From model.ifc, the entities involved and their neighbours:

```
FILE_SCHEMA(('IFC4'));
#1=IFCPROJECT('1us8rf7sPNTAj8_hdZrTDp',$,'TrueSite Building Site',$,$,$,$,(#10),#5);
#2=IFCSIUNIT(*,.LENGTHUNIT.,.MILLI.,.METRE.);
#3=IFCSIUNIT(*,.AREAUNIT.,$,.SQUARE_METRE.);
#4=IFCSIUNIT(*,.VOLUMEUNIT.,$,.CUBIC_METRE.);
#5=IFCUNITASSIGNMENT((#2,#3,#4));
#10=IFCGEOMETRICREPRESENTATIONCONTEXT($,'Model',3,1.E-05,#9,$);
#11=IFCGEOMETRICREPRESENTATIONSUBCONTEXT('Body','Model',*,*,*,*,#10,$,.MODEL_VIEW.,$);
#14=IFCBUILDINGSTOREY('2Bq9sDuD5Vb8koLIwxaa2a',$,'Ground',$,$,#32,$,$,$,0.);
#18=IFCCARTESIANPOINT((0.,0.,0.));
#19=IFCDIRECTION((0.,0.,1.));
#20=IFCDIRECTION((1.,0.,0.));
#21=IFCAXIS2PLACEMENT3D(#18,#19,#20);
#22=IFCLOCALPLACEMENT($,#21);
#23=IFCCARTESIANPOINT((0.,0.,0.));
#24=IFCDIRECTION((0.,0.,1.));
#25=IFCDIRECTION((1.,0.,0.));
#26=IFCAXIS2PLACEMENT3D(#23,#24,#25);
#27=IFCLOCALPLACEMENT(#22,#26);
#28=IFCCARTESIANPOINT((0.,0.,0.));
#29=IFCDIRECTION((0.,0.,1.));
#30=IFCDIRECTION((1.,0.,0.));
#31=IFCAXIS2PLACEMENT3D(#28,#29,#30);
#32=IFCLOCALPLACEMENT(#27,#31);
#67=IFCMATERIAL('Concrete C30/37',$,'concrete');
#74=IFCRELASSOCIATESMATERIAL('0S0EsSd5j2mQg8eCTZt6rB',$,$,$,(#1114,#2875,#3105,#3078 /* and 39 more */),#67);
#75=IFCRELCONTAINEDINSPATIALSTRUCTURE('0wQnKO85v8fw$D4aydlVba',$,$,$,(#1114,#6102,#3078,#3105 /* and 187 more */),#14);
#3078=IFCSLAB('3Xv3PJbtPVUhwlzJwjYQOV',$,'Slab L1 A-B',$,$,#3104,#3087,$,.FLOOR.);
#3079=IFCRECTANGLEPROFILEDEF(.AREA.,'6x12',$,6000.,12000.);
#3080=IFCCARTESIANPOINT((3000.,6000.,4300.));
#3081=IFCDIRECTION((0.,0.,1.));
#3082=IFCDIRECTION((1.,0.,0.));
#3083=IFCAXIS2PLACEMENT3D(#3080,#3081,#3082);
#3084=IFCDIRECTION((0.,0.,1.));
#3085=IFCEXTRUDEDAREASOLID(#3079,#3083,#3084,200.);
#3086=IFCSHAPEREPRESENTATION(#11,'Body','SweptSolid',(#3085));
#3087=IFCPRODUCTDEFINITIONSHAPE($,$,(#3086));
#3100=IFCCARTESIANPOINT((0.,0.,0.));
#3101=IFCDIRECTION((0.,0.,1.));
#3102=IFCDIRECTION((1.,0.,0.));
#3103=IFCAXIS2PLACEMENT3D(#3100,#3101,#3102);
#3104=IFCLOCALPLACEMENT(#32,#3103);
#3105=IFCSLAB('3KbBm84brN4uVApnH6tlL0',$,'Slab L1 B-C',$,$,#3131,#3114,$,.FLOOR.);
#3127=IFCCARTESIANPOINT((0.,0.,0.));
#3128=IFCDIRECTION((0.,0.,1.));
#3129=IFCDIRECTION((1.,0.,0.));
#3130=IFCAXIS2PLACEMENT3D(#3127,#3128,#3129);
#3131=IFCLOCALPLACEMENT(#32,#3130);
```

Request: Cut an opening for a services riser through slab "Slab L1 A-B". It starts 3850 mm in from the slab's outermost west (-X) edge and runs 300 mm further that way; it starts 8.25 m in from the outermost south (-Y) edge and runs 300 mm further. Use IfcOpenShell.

```python
import numpy as np
import ifcopenshell
import ifcopenshell.api.feature
import ifcopenshell.api.geometry
import ifcopenshell.api.root
import ifcopenshell.geom
import ifcopenshell.util.placement
import ifcopenshell.util.representation
import ifcopenshell.util.shape
import ifcopenshell.util.unit

model = ifcopenshell.open("model.ifc")
unit_scale = ifcopenshell.util.unit.calculate_unit_scale(model)
settings = ifcopenshell.geom.settings()


def volume(element):
    """Net volume in cubic metres, openings subtracted."""
    shape = ifcopenshell.geom.create_shape(settings, element)
    return ifcopenshell.util.shape.get_volume(shape.geometry)


slab = model.by_guid("3Xv3PJbtPVUhwlzJwjYQOV")
before = volume(slab)

# Extent in the slab's own axes, in metres. The edges named are its -X and -Y sides.
slab_shape = ifcopenshell.geom.create_shape(settings, slab)
vertices = ifcopenshell.util.shape.get_vertices(slab_shape.geometry)
x_min, y_min, bottom = vertices.min(axis=0)
top = vertices[:, 2].max()

opening = ifcopenshell.api.root.create_entity(model, ifc_class="IfcOpeningElement", name="Services riser opening", predefined_type="OPENING")
context = ifcopenshell.util.representation.get_context(model, "Model", "Body", "MODEL_VIEW")
width, depth = 0.3, 0.3
outline = [(0.0, 0.0), (width, 0.0), (width, depth), (0.0, depth), (0.0, 0.0)]
# Overshoot both faces by 50 mm so the cut is clean.
shape = ifcopenshell.api.geometry.add_slab_representation(
    model, context=context, depth=top - bottom + 0.1, polyline=outline
)
ifcopenshell.api.geometry.assign_representation(model, product=opening, representation=shape)

matrix = ifcopenshell.util.placement.get_local_placement(slab.ObjectPlacement)
matrix[:, 3] = matrix @ np.append(np.array([x_min + 3.85, y_min + 8.25, bottom - 0.05]) / unit_scale, 1.0)
ifcopenshell.api.geometry.edit_object_placement(model, product=opening, matrix=matrix, is_si=False)
ifcopenshell.api.feature.add_feature(model, feature=opening, element=slab)

after = volume(slab)

print(f"slab volume {before:.3f} -> {after:.3f} m3")

model.write("model_edited.ifc")
```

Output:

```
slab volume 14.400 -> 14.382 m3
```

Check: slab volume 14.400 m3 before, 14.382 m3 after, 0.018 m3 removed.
